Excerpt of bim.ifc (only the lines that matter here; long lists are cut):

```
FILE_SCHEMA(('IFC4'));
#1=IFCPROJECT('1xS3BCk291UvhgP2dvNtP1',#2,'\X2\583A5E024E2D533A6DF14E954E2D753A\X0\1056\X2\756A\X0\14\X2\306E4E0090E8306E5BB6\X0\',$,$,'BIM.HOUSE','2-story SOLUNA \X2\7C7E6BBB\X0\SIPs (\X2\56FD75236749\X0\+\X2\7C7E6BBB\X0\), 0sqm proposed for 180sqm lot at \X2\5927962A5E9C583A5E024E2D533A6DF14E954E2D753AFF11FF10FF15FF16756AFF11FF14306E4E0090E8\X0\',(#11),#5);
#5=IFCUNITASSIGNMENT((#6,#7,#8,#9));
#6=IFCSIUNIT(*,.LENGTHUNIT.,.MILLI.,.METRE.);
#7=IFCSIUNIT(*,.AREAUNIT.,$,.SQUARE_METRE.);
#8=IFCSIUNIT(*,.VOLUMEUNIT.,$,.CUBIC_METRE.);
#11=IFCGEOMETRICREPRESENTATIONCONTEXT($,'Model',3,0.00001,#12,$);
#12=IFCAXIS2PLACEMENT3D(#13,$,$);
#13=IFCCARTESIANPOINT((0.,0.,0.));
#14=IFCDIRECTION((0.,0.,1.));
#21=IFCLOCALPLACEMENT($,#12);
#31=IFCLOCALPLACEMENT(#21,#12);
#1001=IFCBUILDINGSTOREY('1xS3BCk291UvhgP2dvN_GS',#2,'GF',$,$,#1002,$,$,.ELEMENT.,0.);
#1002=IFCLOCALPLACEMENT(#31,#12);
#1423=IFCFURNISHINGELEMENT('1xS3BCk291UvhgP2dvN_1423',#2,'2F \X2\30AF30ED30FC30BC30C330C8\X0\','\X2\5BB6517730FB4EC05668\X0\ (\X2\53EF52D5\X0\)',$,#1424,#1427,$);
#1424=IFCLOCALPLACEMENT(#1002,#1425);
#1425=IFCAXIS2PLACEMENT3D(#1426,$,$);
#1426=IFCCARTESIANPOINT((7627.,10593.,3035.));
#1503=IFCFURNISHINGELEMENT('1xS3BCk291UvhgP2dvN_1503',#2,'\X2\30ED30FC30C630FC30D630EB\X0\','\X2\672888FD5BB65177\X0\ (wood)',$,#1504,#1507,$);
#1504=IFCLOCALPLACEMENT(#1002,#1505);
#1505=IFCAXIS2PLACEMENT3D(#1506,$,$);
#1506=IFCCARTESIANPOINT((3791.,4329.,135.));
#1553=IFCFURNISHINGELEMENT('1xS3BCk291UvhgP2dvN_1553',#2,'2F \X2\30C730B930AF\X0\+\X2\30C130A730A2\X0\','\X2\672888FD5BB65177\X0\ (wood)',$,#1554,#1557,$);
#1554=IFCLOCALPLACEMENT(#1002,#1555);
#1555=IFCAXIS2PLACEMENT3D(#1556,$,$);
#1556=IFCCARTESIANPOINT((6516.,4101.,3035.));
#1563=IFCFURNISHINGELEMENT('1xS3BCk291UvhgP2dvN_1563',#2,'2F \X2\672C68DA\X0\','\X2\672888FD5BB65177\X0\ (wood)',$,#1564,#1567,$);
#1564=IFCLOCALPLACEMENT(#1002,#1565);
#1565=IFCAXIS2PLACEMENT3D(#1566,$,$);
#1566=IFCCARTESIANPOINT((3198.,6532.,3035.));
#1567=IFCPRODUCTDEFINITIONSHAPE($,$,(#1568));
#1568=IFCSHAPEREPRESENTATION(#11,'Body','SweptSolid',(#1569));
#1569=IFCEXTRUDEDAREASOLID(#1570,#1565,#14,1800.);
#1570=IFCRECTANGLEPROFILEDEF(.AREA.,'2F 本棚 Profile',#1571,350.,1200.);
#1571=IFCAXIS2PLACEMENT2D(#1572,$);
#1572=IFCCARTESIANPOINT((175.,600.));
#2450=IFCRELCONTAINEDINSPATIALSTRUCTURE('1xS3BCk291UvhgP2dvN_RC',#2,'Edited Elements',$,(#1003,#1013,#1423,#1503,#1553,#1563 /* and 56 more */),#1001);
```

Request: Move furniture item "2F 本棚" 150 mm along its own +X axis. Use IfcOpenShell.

```python
import ifcopenshell
import ifcopenshell.api.geometry
import ifcopenshell.util.placement

model = ifcopenshell.open("bim.ifc")

item = model.by_id(1563)
matrix = ifcopenshell.util.placement.get_local_placement(item.ObjectPlacement)
matrix[:3, 3] += matrix[:3, 0] * 150.0
ifcopenshell.api.geometry.edit_object_placement(model, product=item, matrix=matrix, is_si=False)

print(ifcopenshell.util.placement.get_local_placement(item.ObjectPlacement).round(3) + 0.0)

model.write("bim_v2.ifc")
```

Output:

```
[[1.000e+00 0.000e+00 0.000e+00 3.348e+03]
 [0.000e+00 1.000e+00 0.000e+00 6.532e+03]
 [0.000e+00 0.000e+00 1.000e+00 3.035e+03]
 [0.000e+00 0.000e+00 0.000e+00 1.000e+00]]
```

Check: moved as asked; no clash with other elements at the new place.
